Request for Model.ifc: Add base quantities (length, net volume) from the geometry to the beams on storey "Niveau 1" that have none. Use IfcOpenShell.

First a look at what the model holds.

```python
import ifcopenshell
import ifcopenshell.util.element
import ifcopenshell.util.unit

model = ifcopenshell.open("Model.ifc")
print(model.schema)
for unit_type in ("LENGTHUNIT", "AREAUNIT", "VOLUMEUNIT"):
    print(unit_type, ifcopenshell.util.unit.calculate_unit_scale(model, unit_type))
storey = next(s for s in model.by_type("IfcBuildingStorey") if s.Name == "Niveau 1")
beams = [e for e in ifcopenshell.util.element.get_decomposition(storey) if e.is_a("IfcBeam")]
for e in sorted(beams, key=lambda e: e.id()):
    print(e.id(), e.is_a(), e.Name, list(ifcopenshell.util.element.get_psets(e, qtos_only=True)), sep=" | ")
```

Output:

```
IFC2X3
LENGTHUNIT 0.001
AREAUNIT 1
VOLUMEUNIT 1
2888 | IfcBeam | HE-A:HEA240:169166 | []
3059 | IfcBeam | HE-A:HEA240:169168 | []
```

```python
import ifcopenshell
import ifcopenshell.api.pset
import ifcopenshell.geom
import ifcopenshell.util.element
import ifcopenshell.util.shape
import ifcopenshell.util.unit

model = ifcopenshell.open("Model.ifc")
unit_scale = ifcopenshell.util.unit.calculate_unit_scale(model)
volume_scale = ifcopenshell.util.unit.calculate_unit_scale(model, "VOLUMEUNIT")
settings = ifcopenshell.geom.settings()

storey = next(s for s in model.by_type("IfcBuildingStorey") if s.Name == "Niveau 1")
beams = [e for e in ifcopenshell.util.element.get_decomposition(storey) if e.is_a("IfcBeam")]

for e in sorted(beams, key=lambda e: e.id()):
    if ifcopenshell.util.element.get_psets(e, qtos_only=True, should_inherit=False):
        continue
    # Geometry comes back in metres, in the element's own axes.
    shape = ifcopenshell.geom.create_shape(settings, e)
    values = {
        "Length": ifcopenshell.util.shape.get_max_xyz(shape.geometry) / unit_scale,
        "NetVolume": ifcopenshell.util.shape.get_volume(shape.geometry) / volume_scale,
    }
    qto = ifcopenshell.api.pset.add_qto(model, product=e, name="BaseQuantities")
    ifcopenshell.api.pset.edit_qto(model, qto=qto, properties=values)
    print(e.id(), {k: round(v, 3) for k, v in values.items()})

model.write("Model_updated.ifc")
```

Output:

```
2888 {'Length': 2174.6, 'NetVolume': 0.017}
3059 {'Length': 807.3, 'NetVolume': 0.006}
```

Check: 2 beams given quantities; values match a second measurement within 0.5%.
